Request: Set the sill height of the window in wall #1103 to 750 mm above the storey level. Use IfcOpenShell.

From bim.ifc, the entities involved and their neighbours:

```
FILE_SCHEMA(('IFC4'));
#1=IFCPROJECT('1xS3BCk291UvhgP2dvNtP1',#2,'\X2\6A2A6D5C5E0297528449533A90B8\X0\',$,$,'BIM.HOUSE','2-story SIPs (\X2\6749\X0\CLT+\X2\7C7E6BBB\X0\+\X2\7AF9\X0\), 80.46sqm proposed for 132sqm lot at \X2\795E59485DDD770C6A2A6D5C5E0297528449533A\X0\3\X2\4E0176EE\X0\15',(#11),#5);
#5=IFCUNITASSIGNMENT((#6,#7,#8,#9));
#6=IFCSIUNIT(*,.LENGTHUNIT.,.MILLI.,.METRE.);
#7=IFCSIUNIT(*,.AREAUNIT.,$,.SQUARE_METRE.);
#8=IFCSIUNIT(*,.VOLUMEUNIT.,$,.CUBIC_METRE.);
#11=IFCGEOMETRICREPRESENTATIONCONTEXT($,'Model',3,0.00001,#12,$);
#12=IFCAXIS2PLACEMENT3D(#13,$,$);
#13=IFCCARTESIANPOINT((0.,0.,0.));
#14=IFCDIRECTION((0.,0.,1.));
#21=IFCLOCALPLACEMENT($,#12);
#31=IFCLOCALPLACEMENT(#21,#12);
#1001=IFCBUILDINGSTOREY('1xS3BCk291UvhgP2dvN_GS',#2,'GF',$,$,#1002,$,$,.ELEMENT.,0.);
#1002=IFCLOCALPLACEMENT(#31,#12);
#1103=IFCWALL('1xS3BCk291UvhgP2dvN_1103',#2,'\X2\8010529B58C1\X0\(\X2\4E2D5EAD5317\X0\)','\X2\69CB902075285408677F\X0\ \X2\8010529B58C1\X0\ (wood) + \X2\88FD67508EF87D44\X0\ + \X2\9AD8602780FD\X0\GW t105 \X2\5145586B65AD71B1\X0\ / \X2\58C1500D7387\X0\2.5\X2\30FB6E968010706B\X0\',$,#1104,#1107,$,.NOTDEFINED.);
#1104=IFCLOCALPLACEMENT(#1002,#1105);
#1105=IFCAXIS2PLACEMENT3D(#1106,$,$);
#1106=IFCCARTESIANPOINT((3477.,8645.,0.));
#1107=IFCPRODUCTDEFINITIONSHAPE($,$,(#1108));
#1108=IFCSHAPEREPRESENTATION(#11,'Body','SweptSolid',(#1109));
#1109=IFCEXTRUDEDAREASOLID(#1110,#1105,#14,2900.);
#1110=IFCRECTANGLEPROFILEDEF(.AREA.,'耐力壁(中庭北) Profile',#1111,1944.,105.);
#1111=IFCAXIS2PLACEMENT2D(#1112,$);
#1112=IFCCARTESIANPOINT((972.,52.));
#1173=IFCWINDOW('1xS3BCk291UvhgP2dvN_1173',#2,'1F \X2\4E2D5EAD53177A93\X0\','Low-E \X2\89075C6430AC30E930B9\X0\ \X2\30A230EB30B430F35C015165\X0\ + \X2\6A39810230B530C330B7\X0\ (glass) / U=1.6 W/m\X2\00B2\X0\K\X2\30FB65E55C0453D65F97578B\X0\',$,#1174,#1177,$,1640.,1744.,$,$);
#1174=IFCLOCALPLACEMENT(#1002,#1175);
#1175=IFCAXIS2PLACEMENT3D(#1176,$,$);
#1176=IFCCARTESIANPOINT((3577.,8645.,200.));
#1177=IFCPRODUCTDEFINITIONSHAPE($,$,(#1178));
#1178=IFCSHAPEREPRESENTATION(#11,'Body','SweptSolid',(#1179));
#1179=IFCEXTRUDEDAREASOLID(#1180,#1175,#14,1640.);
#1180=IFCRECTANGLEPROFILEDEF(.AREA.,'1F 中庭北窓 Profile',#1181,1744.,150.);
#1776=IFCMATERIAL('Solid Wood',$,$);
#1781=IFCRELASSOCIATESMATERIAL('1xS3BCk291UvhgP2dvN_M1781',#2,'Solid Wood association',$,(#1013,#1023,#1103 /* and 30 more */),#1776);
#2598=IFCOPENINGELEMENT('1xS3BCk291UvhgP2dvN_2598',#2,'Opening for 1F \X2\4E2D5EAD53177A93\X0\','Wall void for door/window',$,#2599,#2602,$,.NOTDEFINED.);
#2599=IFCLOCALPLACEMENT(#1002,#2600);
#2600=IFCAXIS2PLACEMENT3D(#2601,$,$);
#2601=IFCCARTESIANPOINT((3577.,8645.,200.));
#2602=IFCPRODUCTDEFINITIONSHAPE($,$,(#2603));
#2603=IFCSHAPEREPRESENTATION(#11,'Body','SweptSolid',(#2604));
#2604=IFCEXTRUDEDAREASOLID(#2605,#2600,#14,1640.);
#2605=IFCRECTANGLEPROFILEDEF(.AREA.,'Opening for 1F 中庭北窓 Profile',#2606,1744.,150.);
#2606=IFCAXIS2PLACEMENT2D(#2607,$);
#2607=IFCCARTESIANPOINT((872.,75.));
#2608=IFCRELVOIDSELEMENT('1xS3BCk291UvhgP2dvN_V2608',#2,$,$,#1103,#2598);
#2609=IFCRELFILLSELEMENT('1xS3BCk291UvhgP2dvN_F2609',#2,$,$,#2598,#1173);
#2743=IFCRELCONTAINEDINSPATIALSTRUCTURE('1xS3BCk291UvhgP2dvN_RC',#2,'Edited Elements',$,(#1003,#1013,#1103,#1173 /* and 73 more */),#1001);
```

```python
import numpy as np
import ifcopenshell
import ifcopenshell.api.geometry
import ifcopenshell.geom
import ifcopenshell.util.element
import ifcopenshell.util.placement
import ifcopenshell.util.shape
import ifcopenshell.util.unit

model = ifcopenshell.open("bim.ifc")
unit_scale = ifcopenshell.util.unit.calculate_unit_scale(model)

window = model.by_id(1173)
opening = window.FillsVoids[0].RelatingOpeningElement
storey = ifcopenshell.util.element.get_container(window, ifc_class="IfcBuildingStorey")
level = ifcopenshell.util.placement.get_local_placement(storey.ObjectPlacement)[2, 3]

# The opening's origin need not be at the sill, so measure its lowest point.
shape = ifcopenshell.geom.create_shape(ifcopenshell.geom.settings(), opening)
bottom = ifcopenshell.util.shape.get_shape_bottom_elevation(shape, shape.geometry) / unit_scale
dz = level + 0.75 / unit_scale - bottom

shift = np.array([0.0, 0.0, dz])
# The window is not placed relative to its opening, so move both.
for product in (opening, window):
    matrix = ifcopenshell.util.placement.get_local_placement(product.ObjectPlacement)
    matrix[:3, 3] += shift
    ifcopenshell.api.geometry.edit_object_placement(model, product=product, matrix=matrix, is_si=False)

print(f"moved by {dz * unit_scale:+.3f} m")

model.write("bim_v2.ifc")
```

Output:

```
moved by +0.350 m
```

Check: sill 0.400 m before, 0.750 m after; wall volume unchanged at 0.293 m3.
